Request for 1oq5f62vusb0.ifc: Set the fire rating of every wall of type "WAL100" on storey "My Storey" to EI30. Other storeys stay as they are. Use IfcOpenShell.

First a look at what the model holds.

```python
import ifcopenshell
import ifcopenshell.util.element

model = ifcopenshell.open("1oq5f62vusb0.ifc")
print(model.schema)
storey = next(s for s in model.by_type("IfcBuildingStorey") if s.Name == "My Storey")
walls = [e for e in ifcopenshell.util.element.get_decomposition(storey) if e.is_a("IfcWall")]
seen = {}
for e in walls:
    element_type = ifcopenshell.util.element.get_type(e)
    key = (element_type.Name if element_type != e and element_type else None, ifcopenshell.util.element.get_pset(e, "Pset_WallCommon", "FireRating"))
    seen[key] = seen.get(key, 0) + 1
for (name, value), count in sorted(seen.items(), key=str):
    print(count, "x", name, "|", value)
```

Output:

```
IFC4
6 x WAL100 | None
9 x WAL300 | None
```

```python
import ifcopenshell
import ifcopenshell.api.pset
import ifcopenshell.util.element

model = ifcopenshell.open("1oq5f62vusb0.ifc")

storey = next(s for s in model.by_type("IfcBuildingStorey") if s.Name == "My Storey")
walls = [e for e in ifcopenshell.util.element.get_decomposition(storey) if e.is_a("IfcWall")]

count = 0
for e in walls:
    element_type = ifcopenshell.util.element.get_type(e)
    if element_type in (None, e) or element_type.Name != "WAL100":
        continue
    # add_pset returns the element's existing set when there is one.
    pset = ifcopenshell.api.pset.add_pset(model, product=e, name="Pset_WallCommon")
    ifcopenshell.api.pset.edit_pset(model, pset=pset, properties={"FireRating": "EI30"})
    count += 1

print(count, "walls updated")

model.write("1oq5f62vusb0-out.ifc")
```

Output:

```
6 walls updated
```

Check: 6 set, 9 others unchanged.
